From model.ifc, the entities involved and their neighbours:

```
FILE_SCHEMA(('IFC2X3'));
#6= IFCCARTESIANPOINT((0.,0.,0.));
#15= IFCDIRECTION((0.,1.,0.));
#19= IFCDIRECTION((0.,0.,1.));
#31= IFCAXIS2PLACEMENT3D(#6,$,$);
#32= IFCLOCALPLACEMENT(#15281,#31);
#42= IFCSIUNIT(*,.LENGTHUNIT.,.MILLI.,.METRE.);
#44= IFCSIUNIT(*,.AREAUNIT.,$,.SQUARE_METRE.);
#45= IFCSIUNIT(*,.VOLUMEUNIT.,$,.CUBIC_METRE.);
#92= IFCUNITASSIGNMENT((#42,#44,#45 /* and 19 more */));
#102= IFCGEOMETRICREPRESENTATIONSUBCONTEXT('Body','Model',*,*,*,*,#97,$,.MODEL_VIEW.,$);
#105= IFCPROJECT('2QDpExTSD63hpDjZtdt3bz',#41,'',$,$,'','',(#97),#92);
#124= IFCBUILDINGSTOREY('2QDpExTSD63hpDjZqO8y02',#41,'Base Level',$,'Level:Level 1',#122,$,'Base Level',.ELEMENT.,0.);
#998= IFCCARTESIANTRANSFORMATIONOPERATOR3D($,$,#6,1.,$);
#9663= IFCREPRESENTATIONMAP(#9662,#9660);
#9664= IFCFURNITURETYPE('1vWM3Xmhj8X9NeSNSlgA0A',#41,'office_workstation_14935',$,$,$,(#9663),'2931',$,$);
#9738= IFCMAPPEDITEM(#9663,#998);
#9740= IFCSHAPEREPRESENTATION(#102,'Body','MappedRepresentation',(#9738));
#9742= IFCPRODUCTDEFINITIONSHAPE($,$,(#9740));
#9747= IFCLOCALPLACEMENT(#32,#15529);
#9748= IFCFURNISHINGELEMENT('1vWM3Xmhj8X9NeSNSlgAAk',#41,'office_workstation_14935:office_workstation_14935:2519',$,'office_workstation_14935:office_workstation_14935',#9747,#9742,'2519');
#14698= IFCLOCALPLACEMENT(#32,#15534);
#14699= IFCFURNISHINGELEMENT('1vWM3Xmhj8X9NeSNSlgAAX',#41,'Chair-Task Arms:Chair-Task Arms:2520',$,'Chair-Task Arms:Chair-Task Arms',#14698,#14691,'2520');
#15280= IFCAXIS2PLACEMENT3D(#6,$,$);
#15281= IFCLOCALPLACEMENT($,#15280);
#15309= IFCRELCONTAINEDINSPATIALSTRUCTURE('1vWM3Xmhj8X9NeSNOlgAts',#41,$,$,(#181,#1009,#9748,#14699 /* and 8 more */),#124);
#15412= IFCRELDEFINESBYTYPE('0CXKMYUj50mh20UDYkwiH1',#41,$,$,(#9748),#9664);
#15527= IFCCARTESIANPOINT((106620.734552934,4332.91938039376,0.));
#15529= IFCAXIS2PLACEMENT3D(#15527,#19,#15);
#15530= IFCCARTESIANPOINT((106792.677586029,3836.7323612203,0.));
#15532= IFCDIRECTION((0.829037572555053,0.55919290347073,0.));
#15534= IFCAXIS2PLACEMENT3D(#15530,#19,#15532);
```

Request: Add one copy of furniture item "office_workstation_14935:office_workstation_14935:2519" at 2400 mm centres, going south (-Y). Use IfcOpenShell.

```python
import numpy as np
import ifcopenshell
import ifcopenshell.api.geometry
import ifcopenshell.api.root
import ifcopenshell.util.element
import ifcopenshell.util.placement

model = ifcopenshell.open("model.ifc")


def reuse_history(source, copy):
    """copy_class also copies each property set's owner history, people and application; keep the originals."""
    for rel in copy.IsDefinedBy:
        if rel.is_a("IfcRelDefinesByProperties") and (history := rel.RelatingPropertyDefinition.OwnerHistory):
            rel.RelatingPropertyDefinition.OwnerHistory = source.OwnerHistory
            ifcopenshell.util.element.remove_deep2(model, history)


source = model.by_guid("1vWM3Xmhj8X9NeSNSlgAAk")
base = ifcopenshell.util.placement.get_local_placement(source.ObjectPlacement)
step = np.array([0.0, -1.0, 0.0]) * 2400.0

for i in range(1, 2):
    copy = ifcopenshell.api.root.copy_class(model, product=source)
    copy.Representation = ifcopenshell.util.element.copy_deep(
        model, source.Representation, exclude=["IfcGeometricRepresentationContext", "IfcRepresentationMap"]
    )
    copy.Name = "office_workstation_14935:office_workstation_14935"
    copy.Tag = None
    reuse_history(source, copy)
    matrix = base.copy()
    matrix[:3, 3] += i * step
    print("added at", matrix[:3, 3].round(3) + 0.0)
    ifcopenshell.api.geometry.edit_object_placement(model, product=copy, matrix=matrix, is_si=False)

model.write("model_updated.ifc")
```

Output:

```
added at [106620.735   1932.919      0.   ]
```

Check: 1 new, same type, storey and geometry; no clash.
